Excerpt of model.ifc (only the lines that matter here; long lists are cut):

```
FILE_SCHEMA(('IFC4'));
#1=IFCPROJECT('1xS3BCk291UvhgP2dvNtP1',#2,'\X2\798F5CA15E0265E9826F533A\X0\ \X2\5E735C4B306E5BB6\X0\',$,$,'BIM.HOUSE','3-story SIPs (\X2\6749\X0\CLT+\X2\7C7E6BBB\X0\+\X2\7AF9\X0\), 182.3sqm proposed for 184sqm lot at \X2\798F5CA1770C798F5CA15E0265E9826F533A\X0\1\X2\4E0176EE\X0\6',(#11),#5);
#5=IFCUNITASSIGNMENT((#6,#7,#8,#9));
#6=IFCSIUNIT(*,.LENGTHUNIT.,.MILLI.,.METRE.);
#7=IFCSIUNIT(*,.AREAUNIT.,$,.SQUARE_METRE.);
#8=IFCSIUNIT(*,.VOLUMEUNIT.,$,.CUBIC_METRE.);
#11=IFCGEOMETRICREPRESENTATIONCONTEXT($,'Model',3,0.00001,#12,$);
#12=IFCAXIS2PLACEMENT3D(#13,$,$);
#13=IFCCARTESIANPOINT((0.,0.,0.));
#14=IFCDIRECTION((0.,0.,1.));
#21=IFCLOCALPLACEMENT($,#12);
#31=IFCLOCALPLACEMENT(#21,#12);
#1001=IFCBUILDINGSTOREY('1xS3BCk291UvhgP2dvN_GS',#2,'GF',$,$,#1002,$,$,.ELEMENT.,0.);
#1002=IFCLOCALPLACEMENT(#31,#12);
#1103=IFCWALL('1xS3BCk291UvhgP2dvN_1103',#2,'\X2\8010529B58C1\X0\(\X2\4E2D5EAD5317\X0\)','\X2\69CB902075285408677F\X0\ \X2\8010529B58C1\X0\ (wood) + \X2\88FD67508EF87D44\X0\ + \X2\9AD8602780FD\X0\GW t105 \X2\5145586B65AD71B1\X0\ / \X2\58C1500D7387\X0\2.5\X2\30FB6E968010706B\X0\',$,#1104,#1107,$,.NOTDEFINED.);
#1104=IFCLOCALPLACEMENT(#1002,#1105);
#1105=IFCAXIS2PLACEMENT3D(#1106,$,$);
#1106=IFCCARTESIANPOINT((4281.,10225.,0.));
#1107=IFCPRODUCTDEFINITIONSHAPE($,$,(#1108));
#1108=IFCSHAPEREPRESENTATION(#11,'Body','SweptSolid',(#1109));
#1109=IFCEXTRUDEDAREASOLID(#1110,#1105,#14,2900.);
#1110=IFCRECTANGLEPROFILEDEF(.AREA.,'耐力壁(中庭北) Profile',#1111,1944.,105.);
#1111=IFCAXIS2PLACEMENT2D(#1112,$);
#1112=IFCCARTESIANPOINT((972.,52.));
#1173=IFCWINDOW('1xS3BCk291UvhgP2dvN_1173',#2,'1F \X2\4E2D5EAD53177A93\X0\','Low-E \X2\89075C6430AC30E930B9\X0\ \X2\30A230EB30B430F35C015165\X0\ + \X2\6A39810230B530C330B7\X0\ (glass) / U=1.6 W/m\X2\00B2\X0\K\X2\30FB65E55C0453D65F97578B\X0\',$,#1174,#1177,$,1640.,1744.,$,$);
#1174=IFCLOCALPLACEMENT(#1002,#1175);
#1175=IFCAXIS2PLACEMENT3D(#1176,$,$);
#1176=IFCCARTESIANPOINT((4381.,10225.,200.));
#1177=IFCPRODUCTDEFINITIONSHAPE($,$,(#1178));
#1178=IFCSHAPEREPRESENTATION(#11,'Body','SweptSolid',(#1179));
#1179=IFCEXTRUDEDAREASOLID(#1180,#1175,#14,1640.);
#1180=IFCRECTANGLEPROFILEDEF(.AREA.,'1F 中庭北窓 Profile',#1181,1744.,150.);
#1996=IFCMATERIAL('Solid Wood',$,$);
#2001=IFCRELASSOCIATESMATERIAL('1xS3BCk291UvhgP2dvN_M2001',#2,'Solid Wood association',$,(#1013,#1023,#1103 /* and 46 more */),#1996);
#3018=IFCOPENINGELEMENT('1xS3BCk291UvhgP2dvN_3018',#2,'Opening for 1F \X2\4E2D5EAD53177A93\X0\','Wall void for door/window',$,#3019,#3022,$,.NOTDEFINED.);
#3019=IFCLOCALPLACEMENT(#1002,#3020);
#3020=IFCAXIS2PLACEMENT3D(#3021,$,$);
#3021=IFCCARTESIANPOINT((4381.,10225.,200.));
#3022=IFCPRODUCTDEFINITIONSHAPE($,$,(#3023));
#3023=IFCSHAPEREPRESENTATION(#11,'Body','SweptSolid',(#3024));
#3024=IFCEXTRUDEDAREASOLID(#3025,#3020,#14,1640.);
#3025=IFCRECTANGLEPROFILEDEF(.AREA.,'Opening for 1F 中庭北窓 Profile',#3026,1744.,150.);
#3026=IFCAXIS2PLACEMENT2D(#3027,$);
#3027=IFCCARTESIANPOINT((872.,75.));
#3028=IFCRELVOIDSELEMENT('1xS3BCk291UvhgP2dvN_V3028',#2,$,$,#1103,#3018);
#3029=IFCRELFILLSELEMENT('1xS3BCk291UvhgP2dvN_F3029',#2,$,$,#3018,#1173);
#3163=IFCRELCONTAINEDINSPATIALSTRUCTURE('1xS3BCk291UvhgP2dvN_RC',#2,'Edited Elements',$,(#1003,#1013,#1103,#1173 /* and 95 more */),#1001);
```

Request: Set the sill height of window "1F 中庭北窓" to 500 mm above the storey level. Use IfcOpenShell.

```python
import numpy as np
import ifcopenshell
import ifcopenshell.api.geometry
import ifcopenshell.geom
import ifcopenshell.util.element
import ifcopenshell.util.placement
import ifcopenshell.util.shape
import ifcopenshell.util.unit

model = ifcopenshell.open("model.ifc")
unit_scale = ifcopenshell.util.unit.calculate_unit_scale(model)

window = model.by_guid("1xS3BCk291UvhgP2dvN_1173")
opening = window.FillsVoids[0].RelatingOpeningElement
storey = ifcopenshell.util.element.get_container(window, ifc_class="IfcBuildingStorey")
level = ifcopenshell.util.placement.get_local_placement(storey.ObjectPlacement)[2, 3]

# The opening's origin need not be at the sill, so measure its lowest point.
shape = ifcopenshell.geom.create_shape(ifcopenshell.geom.settings(), opening)
bottom = ifcopenshell.util.shape.get_shape_bottom_elevation(shape, shape.geometry) / unit_scale
dz = level + 0.5 / unit_scale - bottom

shift = np.array([0.0, 0.0, dz])
# The window is not placed relative to its opening, so move both.
for product in (opening, window):
    matrix = ifcopenshell.util.placement.get_local_placement(product.ObjectPlacement)
    matrix[:3, 3] += shift
    ifcopenshell.api.geometry.edit_object_placement(model, product=product, matrix=matrix, is_si=False)

print(f"moved by {dz * unit_scale:+.3f} m")

model.write("model_rev.ifc")
```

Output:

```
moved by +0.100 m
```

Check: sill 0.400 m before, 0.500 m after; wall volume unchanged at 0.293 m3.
